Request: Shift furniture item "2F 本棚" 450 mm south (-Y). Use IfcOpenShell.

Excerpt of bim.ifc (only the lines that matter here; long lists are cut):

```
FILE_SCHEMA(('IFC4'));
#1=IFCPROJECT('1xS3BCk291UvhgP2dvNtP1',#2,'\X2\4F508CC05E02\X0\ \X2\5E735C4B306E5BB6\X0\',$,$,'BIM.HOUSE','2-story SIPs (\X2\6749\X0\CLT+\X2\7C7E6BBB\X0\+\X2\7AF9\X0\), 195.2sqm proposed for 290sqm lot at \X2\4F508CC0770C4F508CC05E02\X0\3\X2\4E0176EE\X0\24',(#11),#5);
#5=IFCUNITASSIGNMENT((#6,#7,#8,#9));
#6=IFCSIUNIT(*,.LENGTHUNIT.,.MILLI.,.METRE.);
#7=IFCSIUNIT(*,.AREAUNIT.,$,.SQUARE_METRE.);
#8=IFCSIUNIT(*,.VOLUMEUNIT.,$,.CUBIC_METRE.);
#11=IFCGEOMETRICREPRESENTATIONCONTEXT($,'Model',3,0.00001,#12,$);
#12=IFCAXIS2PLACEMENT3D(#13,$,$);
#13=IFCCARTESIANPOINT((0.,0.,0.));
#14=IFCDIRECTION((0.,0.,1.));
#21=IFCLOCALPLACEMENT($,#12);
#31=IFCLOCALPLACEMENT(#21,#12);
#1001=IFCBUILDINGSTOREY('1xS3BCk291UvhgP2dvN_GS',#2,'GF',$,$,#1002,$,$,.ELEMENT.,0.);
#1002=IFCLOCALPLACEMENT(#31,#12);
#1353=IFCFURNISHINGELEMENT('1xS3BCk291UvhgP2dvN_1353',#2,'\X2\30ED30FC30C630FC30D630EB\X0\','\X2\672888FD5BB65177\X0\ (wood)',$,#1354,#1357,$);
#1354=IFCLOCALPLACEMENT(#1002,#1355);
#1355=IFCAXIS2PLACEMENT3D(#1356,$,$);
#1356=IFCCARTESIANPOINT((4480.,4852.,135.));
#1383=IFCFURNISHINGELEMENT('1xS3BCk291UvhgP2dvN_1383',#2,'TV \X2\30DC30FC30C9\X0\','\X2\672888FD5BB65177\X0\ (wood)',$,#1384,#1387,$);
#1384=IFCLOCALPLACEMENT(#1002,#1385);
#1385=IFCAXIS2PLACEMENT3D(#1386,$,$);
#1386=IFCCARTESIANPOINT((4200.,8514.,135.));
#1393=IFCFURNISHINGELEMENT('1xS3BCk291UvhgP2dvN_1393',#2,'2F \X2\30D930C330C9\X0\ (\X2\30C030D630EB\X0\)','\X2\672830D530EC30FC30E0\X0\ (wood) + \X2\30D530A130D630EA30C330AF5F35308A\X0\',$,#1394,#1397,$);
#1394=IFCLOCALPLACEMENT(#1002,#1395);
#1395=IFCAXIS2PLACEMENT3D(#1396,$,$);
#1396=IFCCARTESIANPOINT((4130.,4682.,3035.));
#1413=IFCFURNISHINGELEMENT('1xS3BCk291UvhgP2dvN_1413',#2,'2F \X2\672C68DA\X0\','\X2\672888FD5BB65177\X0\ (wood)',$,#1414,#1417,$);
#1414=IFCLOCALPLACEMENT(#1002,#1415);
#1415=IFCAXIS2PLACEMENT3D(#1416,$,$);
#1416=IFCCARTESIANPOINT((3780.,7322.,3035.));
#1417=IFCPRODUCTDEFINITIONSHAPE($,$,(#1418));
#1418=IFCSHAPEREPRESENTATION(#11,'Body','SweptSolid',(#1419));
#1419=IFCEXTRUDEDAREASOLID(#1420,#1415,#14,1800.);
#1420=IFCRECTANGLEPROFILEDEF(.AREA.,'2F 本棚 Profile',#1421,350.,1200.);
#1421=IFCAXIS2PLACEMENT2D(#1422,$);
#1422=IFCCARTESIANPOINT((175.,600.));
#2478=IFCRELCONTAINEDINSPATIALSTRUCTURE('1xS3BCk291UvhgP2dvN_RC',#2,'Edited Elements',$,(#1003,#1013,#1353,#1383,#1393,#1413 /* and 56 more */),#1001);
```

```python
import ifcopenshell
import ifcopenshell.api.geometry
import ifcopenshell.util.placement

model = ifcopenshell.open("bim.ifc")

item = model.by_guid("1xS3BCk291UvhgP2dvN_1413")
matrix = ifcopenshell.util.placement.get_local_placement(item.ObjectPlacement)
matrix[1, 3] -= 450.0
ifcopenshell.api.geometry.edit_object_placement(model, product=item, matrix=matrix, is_si=False)

print(ifcopenshell.util.placement.get_local_placement(item.ObjectPlacement).round(3) + 0.0)

model.write("bim_edited.ifc")
```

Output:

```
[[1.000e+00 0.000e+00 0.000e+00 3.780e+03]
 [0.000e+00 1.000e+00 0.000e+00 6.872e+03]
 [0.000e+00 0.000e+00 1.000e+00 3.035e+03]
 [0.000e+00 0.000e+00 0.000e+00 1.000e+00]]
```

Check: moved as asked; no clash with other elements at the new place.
